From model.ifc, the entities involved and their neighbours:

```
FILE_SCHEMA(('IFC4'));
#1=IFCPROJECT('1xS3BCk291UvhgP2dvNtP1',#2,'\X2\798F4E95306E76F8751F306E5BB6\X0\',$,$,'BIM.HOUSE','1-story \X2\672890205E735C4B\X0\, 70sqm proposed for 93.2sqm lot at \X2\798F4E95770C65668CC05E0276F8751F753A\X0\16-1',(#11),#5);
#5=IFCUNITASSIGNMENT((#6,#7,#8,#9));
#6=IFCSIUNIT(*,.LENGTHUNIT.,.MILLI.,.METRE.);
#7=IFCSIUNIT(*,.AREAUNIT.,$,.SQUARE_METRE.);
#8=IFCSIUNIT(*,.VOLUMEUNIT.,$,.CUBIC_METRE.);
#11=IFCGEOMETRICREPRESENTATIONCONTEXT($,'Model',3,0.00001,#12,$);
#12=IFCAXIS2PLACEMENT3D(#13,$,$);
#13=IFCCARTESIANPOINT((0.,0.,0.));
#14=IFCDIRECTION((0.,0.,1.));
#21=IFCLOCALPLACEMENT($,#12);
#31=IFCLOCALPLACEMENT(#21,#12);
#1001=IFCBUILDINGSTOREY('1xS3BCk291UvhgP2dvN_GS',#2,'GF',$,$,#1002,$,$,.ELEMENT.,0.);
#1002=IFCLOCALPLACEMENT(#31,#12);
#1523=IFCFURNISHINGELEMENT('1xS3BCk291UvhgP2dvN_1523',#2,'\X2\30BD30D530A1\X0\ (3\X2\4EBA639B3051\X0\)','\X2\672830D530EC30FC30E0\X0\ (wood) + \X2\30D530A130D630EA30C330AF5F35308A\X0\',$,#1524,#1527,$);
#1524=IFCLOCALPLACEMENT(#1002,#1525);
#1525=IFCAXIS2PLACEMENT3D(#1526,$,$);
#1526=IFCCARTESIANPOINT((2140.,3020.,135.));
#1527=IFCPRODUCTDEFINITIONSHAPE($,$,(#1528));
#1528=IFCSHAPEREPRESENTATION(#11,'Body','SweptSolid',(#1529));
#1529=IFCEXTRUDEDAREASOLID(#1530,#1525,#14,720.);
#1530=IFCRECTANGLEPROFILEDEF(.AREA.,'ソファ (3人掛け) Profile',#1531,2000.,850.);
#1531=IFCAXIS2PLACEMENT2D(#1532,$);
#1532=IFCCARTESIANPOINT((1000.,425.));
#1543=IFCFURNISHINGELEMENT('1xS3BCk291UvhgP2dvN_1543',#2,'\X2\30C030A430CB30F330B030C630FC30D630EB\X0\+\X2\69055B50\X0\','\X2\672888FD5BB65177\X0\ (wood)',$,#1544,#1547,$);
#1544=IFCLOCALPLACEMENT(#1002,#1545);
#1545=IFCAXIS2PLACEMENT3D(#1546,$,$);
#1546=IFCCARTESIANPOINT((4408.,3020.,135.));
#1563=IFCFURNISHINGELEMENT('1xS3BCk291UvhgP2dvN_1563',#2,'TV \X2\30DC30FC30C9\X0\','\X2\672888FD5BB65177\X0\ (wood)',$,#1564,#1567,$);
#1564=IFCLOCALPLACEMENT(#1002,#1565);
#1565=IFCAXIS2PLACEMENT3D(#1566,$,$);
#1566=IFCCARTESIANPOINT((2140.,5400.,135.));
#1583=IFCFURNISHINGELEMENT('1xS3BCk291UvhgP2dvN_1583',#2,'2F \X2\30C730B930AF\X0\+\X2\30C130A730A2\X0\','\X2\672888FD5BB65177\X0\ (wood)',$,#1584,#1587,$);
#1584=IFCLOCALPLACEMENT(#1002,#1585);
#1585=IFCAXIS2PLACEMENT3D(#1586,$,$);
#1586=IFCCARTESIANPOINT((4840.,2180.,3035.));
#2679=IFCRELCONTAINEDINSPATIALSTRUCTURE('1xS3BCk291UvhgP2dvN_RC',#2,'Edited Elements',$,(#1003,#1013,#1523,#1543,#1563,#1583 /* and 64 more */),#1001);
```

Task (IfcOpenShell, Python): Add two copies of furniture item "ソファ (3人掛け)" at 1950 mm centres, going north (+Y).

```python
import numpy as np
import ifcopenshell
import ifcopenshell.api.geometry
import ifcopenshell.api.root
import ifcopenshell.util.element
import ifcopenshell.util.placement

model = ifcopenshell.open("model.ifc")


def reuse_history(source, copy):
    """copy_class also copies each property set's owner history, people and application; keep the originals."""
    for rel in copy.IsDefinedBy:
        if rel.is_a("IfcRelDefinesByProperties") and (history := rel.RelatingPropertyDefinition.OwnerHistory):
            rel.RelatingPropertyDefinition.OwnerHistory = source.OwnerHistory
            ifcopenshell.util.element.remove_deep2(model, history)


source = model.by_id(1523)
base = ifcopenshell.util.placement.get_local_placement(source.ObjectPlacement)
step = np.array([0.0, 1.0, 0.0]) * 1950.0

for i in range(1, 3):
    copy = ifcopenshell.api.root.copy_class(model, product=source)
    copy.Representation = ifcopenshell.util.element.copy_deep(
        model, source.Representation, exclude=["IfcGeometricRepresentationContext", "IfcRepresentationMap"]
    )
    reuse_history(source, copy)
    matrix = base.copy()
    matrix[:3, 3] += i * step
    print("added at", matrix[:3, 3].round(3) + 0.0)
    ifcopenshell.api.geometry.edit_object_placement(model, product=copy, matrix=matrix, is_si=False)

model.write("model-out.ifc")
```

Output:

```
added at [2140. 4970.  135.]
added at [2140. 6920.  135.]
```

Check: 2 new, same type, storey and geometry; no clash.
